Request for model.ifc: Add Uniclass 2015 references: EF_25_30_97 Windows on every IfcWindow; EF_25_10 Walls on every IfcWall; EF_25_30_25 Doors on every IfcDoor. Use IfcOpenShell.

First a look at what the model holds.

```python
import ifcopenshell

model = ifcopenshell.open("model.ifc")
print(model.schema)
print("classifications:", [c.Name for c in model.by_type("IfcClassification")])
for ifc_class in ("IfcDoor", "IfcRoof", "IfcStair", "IfcWall", "IfcWindow"):
    print(ifc_class, len(model.by_type(ifc_class)))
```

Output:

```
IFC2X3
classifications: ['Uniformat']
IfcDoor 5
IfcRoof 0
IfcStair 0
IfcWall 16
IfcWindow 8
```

```python
import ifcopenshell
import ifcopenshell.api.classification

model = ifcopenshell.open("model.ifc")

# IFC2X3 requires Source and Edition and has no link from the project to the system.
system = model.create_entity("IfcClassification", Source="NBS", Edition="2015", Name="Uniclass 2015")

codes = {
    "IfcWindow": ("EF_25_30_97", "Windows"),
    "IfcWall": ("EF_25_10", "Walls"),
    "IfcDoor": ("EF_25_30_25", "Doors"),
}
for ifc_class, (code, name) in codes.items():
    products = model.by_type(ifc_class)
    ifcopenshell.api.classification.add_reference(
        model, products=products, classification=system, identification=code, name=name
    )
    print(code, len(products))

model.write("model-out.ifc")
```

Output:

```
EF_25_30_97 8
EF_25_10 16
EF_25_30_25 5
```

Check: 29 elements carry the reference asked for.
